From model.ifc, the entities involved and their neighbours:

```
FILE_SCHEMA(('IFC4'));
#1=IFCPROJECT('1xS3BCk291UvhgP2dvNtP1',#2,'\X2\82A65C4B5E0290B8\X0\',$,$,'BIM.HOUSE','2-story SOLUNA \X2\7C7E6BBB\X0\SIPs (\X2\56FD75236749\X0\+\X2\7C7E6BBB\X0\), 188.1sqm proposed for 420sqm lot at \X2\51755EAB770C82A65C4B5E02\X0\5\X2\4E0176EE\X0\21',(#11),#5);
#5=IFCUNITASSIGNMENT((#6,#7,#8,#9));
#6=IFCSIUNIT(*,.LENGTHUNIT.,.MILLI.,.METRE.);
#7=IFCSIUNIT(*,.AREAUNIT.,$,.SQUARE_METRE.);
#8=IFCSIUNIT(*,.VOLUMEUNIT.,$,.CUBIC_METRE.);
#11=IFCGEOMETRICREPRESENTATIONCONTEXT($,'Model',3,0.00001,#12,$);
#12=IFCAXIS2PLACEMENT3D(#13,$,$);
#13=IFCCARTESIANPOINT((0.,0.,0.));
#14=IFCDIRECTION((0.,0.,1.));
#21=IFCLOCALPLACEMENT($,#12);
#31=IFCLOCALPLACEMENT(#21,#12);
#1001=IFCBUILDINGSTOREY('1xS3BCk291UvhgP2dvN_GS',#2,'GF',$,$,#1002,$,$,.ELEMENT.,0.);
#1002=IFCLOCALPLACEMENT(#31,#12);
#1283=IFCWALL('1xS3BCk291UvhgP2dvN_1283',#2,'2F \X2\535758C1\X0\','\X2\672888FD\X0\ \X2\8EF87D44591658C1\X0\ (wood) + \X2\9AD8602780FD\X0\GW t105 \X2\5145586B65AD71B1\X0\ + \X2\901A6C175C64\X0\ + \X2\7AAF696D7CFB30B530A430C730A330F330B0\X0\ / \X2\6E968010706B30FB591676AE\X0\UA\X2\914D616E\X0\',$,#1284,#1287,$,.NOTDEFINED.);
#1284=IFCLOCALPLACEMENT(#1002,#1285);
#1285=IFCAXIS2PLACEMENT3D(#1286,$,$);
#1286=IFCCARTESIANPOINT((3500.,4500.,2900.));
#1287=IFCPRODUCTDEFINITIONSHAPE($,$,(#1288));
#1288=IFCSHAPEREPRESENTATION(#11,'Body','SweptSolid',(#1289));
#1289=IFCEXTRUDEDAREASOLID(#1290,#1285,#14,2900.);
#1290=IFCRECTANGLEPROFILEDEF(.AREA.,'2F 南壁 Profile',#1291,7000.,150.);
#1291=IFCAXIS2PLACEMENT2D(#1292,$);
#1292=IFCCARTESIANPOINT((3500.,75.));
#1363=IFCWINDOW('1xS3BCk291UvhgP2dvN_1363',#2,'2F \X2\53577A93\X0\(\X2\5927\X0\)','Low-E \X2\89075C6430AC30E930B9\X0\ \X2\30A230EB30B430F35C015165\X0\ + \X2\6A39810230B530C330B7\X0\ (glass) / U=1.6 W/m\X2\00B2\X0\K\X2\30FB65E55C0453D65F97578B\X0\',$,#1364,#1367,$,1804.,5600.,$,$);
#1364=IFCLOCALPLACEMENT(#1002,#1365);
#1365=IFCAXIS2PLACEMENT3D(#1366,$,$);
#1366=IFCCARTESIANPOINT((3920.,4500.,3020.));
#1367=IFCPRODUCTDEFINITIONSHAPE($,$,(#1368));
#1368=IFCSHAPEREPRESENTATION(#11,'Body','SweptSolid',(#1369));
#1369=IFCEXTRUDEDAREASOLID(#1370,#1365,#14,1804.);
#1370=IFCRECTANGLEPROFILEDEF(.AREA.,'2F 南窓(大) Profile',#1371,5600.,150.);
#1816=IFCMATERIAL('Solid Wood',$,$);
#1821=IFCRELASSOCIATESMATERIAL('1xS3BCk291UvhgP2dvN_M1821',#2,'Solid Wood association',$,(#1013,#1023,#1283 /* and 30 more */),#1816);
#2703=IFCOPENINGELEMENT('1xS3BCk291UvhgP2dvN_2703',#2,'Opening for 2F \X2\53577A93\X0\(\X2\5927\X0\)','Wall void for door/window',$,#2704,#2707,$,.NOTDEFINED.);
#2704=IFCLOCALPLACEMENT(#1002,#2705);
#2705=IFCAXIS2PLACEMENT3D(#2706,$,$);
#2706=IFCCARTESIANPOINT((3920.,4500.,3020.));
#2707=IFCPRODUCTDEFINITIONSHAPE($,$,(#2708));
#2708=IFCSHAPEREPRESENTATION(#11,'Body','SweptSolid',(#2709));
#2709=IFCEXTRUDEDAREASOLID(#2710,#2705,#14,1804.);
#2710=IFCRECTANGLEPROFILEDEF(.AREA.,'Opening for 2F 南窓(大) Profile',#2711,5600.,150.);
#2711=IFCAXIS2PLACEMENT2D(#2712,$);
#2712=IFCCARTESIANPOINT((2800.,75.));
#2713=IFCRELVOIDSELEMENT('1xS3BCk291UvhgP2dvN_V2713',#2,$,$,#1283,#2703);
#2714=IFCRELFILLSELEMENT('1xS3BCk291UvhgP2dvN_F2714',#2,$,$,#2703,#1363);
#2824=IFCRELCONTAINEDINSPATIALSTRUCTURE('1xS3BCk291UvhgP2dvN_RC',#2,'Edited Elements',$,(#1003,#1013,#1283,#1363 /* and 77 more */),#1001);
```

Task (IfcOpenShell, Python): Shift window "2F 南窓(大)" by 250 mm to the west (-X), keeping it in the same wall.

```python
import ifcopenshell
import ifcopenshell.api.geometry
import ifcopenshell.util.placement

model = ifcopenshell.open("model.ifc")

window = model.by_guid("1xS3BCk291UvhgP2dvN_1363")
opening = window.FillsVoids[0].RelatingOpeningElement
wall = opening.VoidsElements[0].RelatingBuildingElement

wall_matrix = ifcopenshell.util.placement.get_local_placement(wall.ObjectPlacement)
shift = wall_matrix[:3, 0] * -250.0
before = ifcopenshell.util.placement.get_local_placement(window.ObjectPlacement)[:3, 3].copy()

# The window is not placed relative to its opening, so move both.
for product in (opening, window):
    matrix = ifcopenshell.util.placement.get_local_placement(product.ObjectPlacement)
    matrix[:3, 3] += shift
    ifcopenshell.api.geometry.edit_object_placement(model, product=product, matrix=matrix, is_si=False)

after = ifcopenshell.util.placement.get_local_placement(window.ObjectPlacement)[:3, 3]
print("window moved by", (after - before).round(3) + 0.0)

model.write("model_updated.ifc")
```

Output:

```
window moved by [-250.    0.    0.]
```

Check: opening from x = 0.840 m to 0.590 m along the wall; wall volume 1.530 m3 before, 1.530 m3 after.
